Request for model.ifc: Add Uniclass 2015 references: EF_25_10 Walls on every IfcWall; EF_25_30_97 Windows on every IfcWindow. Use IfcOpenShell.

First a look at what the model holds.

```python
import ifcopenshell

model = ifcopenshell.open("model.ifc")
print(model.schema)
print("classifications:", [c.Name for c in model.by_type("IfcClassification")])
for ifc_class in ("IfcDoor", "IfcRoof", "IfcStair", "IfcWall", "IfcWindow"):
    print(ifc_class, len(model.by_type(ifc_class)))
```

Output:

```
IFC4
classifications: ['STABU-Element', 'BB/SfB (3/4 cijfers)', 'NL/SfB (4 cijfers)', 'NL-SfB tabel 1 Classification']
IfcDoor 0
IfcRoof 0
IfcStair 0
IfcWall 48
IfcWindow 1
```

```python
import ifcopenshell
import ifcopenshell.api.classification

model = ifcopenshell.open("model.ifc")

system = ifcopenshell.api.classification.add_classification(model, classification="Uniclass 2015")

codes = {
    "IfcWall": ("EF_25_10", "Walls"),
    "IfcWindow": ("EF_25_30_97", "Windows"),
}
for ifc_class, (code, name) in codes.items():
    products = model.by_type(ifc_class)
    ifcopenshell.api.classification.add_reference(
        model, products=products, classification=system, identification=code, name=name
    )
    print(code, len(products))

model.write("model-out.ifc")
```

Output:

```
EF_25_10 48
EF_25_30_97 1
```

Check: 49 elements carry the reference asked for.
